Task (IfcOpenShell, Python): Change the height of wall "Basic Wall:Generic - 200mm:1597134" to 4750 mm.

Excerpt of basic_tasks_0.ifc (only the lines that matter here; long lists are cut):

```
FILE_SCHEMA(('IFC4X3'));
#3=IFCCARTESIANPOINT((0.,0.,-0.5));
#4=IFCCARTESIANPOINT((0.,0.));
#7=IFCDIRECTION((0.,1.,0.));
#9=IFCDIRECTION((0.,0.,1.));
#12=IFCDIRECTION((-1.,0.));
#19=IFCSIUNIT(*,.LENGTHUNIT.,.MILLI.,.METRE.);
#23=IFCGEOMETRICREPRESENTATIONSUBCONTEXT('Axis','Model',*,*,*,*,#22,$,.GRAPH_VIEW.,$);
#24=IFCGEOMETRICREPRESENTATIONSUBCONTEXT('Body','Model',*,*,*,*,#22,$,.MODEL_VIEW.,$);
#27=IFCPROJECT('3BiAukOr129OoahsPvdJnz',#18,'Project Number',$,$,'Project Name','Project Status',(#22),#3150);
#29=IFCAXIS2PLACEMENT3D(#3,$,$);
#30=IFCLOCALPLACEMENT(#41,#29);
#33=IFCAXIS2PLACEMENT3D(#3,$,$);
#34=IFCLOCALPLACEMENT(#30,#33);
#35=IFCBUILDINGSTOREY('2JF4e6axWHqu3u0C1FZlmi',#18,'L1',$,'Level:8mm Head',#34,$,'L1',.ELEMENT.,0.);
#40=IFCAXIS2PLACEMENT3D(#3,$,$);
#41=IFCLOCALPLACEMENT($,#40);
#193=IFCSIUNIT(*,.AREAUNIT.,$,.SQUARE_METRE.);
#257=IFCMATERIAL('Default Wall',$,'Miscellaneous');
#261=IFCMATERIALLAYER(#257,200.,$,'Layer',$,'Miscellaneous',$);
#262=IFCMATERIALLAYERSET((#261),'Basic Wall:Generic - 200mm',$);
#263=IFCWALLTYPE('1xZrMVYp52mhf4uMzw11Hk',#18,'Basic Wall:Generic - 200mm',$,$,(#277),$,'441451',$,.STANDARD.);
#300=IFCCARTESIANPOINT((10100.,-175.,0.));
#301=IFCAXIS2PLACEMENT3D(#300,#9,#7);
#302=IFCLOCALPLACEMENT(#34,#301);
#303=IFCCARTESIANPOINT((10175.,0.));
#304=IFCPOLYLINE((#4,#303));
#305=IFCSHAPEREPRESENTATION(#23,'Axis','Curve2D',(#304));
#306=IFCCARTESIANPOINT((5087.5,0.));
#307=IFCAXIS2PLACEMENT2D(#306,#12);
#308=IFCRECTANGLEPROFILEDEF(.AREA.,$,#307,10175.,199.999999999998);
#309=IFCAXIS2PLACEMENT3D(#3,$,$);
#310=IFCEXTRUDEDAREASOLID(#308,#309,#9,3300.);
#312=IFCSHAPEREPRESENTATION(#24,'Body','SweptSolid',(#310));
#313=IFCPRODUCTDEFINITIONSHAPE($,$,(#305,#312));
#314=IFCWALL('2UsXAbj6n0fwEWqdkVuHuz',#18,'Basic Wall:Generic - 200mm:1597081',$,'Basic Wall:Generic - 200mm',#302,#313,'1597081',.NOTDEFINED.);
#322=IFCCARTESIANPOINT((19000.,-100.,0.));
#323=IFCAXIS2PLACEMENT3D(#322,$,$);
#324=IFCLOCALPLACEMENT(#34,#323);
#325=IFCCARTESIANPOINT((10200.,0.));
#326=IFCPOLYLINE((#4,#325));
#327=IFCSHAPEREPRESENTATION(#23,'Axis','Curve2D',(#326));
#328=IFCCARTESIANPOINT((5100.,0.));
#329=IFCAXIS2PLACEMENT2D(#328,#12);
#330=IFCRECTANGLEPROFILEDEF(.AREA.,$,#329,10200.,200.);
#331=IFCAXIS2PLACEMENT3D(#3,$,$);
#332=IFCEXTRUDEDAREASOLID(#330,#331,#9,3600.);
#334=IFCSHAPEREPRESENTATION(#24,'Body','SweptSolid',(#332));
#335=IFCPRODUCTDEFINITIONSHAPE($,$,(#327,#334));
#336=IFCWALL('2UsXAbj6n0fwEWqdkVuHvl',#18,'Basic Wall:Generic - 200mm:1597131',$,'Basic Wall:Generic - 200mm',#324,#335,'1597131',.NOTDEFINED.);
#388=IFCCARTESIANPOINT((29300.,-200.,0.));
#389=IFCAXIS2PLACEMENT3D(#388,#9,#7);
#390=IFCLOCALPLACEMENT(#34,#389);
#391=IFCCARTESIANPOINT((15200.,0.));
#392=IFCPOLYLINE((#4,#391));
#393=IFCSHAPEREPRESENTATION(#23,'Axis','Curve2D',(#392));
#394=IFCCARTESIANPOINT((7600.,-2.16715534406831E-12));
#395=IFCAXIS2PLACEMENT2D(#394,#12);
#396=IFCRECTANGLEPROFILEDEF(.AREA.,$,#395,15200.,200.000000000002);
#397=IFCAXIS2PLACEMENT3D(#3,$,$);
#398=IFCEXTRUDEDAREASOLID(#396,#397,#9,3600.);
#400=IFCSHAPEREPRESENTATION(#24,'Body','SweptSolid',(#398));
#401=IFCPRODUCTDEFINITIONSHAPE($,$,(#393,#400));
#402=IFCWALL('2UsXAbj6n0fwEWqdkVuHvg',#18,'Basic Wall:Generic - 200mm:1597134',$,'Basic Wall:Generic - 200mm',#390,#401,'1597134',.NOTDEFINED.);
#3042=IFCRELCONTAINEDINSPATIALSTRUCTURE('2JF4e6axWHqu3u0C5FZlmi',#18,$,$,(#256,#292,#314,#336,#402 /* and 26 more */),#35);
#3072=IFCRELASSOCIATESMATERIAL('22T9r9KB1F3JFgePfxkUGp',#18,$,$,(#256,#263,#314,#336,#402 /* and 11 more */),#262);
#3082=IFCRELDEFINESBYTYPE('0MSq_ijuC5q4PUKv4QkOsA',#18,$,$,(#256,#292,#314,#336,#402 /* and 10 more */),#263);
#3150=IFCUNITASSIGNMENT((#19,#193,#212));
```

```python
import ifcopenshell
import ifcopenshell.geom
import ifcopenshell.util.representation
import ifcopenshell.util.shape
import ifcopenshell.util.unit

model = ifcopenshell.open("basic_tasks_0.ifc")
unit_scale = ifcopenshell.util.unit.calculate_unit_scale(model)
settings = ifcopenshell.geom.settings()


def volume(element):
    """Net volume in cubic metres, openings subtracted."""
    shape = ifcopenshell.geom.create_shape(settings, element)
    return ifcopenshell.util.shape.get_volume(shape.geometry)


wall = model.by_guid("2UsXAbj6n0fwEWqdkVuHvg")
before = volume(wall)

body = ifcopenshell.util.representation.get_representation(wall, "Model", "Body")
solid = body.Items[0]
old_height = solid.Depth
solid.Depth = 4.75 / unit_scale
after = volume(wall)

print(f"height {old_height:g} -> {solid.Depth:g}, volume {before:.3f} -> {after:.3f} m3")

model.write("basic_tasks_0_updated.ifc")
```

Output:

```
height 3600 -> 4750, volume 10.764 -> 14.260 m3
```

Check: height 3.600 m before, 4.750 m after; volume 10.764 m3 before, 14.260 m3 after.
